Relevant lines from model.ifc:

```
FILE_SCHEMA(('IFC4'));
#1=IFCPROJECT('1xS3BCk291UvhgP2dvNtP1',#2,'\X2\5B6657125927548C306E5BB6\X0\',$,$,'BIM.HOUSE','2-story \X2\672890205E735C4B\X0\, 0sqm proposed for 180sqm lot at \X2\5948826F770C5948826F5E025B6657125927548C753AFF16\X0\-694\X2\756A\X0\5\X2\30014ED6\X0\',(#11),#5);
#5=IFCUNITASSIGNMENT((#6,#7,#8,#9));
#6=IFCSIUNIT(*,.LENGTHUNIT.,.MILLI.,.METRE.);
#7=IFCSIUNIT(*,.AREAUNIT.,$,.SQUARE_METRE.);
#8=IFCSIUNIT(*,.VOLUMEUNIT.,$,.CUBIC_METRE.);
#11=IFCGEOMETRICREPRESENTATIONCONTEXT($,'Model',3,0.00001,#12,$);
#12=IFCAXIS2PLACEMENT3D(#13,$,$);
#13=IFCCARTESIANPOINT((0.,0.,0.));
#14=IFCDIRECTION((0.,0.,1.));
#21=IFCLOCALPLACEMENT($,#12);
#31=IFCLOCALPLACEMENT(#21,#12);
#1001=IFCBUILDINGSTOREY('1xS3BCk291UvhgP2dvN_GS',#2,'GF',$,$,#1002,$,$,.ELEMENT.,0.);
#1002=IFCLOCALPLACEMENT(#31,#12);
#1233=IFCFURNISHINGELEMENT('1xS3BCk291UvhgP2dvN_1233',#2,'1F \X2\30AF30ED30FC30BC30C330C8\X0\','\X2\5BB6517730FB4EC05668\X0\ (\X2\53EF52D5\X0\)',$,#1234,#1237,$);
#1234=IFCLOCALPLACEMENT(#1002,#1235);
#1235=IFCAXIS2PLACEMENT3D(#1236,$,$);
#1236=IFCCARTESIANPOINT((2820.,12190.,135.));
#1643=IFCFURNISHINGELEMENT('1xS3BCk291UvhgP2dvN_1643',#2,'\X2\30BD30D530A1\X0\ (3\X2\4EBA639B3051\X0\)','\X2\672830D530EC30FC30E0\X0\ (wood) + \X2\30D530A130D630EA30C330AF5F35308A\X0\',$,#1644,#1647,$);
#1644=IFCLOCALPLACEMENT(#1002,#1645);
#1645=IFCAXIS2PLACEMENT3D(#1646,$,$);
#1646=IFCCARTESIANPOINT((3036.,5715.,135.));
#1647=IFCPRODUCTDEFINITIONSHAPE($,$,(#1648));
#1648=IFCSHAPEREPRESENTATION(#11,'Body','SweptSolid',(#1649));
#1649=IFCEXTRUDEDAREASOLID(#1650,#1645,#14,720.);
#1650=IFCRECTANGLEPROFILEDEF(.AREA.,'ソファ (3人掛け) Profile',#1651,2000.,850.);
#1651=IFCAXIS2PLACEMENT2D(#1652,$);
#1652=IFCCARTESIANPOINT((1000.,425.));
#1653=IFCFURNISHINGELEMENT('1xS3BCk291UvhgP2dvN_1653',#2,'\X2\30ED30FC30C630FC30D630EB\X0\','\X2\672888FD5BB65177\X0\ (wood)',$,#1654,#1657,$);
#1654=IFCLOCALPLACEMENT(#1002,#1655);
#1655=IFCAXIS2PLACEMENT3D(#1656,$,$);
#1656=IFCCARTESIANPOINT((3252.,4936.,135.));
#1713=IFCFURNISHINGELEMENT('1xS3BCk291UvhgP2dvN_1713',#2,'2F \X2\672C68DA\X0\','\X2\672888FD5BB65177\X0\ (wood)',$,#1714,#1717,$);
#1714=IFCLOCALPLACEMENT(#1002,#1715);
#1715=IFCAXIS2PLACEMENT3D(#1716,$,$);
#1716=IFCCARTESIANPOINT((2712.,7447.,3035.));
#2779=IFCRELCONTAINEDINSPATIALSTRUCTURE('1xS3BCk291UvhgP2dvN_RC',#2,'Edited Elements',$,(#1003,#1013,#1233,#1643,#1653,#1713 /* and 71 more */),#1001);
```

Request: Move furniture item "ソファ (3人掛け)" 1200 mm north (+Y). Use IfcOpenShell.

```python
import ifcopenshell
import ifcopenshell.api.geometry
import ifcopenshell.util.placement
import ifcopenshell.util.unit

model = ifcopenshell.open("model.ifc")
unit_scale = ifcopenshell.util.unit.calculate_unit_scale(model)

item = model.by_id(1643)
matrix = ifcopenshell.util.placement.get_local_placement(item.ObjectPlacement)
matrix[1, 3] += 1.2 / unit_scale
ifcopenshell.api.geometry.edit_object_placement(model, product=item, matrix=matrix, is_si=False)

print(ifcopenshell.util.placement.get_local_placement(item.ObjectPlacement).round(3) + 0.0)

model.write("model_rev.ifc")
```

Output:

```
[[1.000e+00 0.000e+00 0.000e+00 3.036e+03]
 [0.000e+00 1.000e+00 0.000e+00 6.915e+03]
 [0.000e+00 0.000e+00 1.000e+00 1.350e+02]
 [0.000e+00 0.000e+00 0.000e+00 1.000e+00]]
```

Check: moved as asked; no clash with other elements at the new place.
